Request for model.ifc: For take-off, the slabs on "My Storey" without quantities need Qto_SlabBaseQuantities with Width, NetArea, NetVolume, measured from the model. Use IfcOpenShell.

First a look at what the model holds.

```python
import ifcopenshell
import ifcopenshell.util.element
import ifcopenshell.util.unit

model = ifcopenshell.open("model.ifc")
print(model.schema)
for unit_type in ("LENGTHUNIT", "AREAUNIT", "VOLUMEUNIT"):
    print(unit_type, ifcopenshell.util.unit.calculate_unit_scale(model, unit_type))
storey = next(s for s in model.by_type("IfcBuildingStorey") if s.Name == "My Storey")
slabs = [e for e in ifcopenshell.util.element.get_decomposition(storey) if e.is_a("IfcSlab")]
for e in sorted(slabs, key=lambda e: e.id()):
    print(e.id(), e.is_a(), e.Name, list(ifcopenshell.util.element.get_psets(e, qtos_only=True)), sep=" | ")
```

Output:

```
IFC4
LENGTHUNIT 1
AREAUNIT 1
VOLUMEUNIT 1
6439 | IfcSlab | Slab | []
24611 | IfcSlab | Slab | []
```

```python
import ifcopenshell
import ifcopenshell.api.pset
import ifcopenshell.geom
import ifcopenshell.util.element
import ifcopenshell.util.shape
import ifcopenshell.util.unit

model = ifcopenshell.open("model.ifc")
unit_scale = ifcopenshell.util.unit.calculate_unit_scale(model)
area_scale = ifcopenshell.util.unit.calculate_unit_scale(model, "AREAUNIT")
volume_scale = ifcopenshell.util.unit.calculate_unit_scale(model, "VOLUMEUNIT")
settings = ifcopenshell.geom.settings()

storey = next(s for s in model.by_type("IfcBuildingStorey") if s.Name == "My Storey")
slabs = [e for e in ifcopenshell.util.element.get_decomposition(storey) if e.is_a("IfcSlab")]

for e in sorted(slabs, key=lambda e: e.id()):
    if ifcopenshell.util.element.get_psets(e, qtos_only=True, should_inherit=False):
        continue
    # Geometry comes back in metres, in the element's own axes.
    shape = ifcopenshell.geom.create_shape(settings, e)
    values = {
        "Width": ifcopenshell.util.shape.get_z(shape.geometry) / unit_scale,
        "NetArea": ifcopenshell.util.shape.get_footprint_area(shape.geometry) / area_scale,
        "NetVolume": ifcopenshell.util.shape.get_volume(shape.geometry) / volume_scale,
    }
    qto = ifcopenshell.api.pset.add_qto(model, product=e, name="Qto_SlabBaseQuantities")
    ifcopenshell.api.pset.edit_qto(model, qto=qto, properties=values)
    print(e.id(), {k: round(v, 3) for k, v in values.items()})

model.write("model_rev.ifc")
```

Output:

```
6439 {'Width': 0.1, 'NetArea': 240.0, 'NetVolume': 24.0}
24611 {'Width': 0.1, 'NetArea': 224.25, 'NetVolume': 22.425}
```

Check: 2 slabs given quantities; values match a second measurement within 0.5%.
